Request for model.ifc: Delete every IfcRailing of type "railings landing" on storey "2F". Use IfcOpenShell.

First a look at what the model holds.

```python
import ifcopenshell
import ifcopenshell.util.element

model = ifcopenshell.open("model.ifc")
print(model.schema)
storey = next(s for s in model.by_type("IfcBuildingStorey") if s.Name == "2F")
railings = [e for e in ifcopenshell.util.element.get_decomposition(storey) if e.is_a("IfcRailing")]
seen = {}
for e in railings:
    element_type = ifcopenshell.util.element.get_type(e)
    name = element_type.Name if element_type not in (None, e) else None
    seen[name] = seen.get(name, 0) + 1
for name, count in sorted(seen.items(), key=str):
    print(count, "x", name)
```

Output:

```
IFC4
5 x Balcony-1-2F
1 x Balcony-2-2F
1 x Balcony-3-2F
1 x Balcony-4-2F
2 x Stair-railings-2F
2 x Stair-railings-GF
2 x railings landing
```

```python
import ifcopenshell
import ifcopenshell.api.root
import ifcopenshell.util.element

model = ifcopenshell.open("model.ifc")

storey = next(s for s in model.by_type("IfcBuildingStorey") if s.Name == "2F")
railings = [e for e in ifcopenshell.util.element.get_decomposition(storey) if e.is_a("IfcRailing")]
targets = [e for e in railings if (t := ifcopenshell.util.element.get_type(e)) not in (None, e) and t.Name == "railings landing"]

for e in targets:
    ifcopenshell.api.root.remove_product(model, product=e)
print(len(targets), "removed")

model.write("model_updated.ifc")
```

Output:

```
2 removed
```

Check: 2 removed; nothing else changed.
